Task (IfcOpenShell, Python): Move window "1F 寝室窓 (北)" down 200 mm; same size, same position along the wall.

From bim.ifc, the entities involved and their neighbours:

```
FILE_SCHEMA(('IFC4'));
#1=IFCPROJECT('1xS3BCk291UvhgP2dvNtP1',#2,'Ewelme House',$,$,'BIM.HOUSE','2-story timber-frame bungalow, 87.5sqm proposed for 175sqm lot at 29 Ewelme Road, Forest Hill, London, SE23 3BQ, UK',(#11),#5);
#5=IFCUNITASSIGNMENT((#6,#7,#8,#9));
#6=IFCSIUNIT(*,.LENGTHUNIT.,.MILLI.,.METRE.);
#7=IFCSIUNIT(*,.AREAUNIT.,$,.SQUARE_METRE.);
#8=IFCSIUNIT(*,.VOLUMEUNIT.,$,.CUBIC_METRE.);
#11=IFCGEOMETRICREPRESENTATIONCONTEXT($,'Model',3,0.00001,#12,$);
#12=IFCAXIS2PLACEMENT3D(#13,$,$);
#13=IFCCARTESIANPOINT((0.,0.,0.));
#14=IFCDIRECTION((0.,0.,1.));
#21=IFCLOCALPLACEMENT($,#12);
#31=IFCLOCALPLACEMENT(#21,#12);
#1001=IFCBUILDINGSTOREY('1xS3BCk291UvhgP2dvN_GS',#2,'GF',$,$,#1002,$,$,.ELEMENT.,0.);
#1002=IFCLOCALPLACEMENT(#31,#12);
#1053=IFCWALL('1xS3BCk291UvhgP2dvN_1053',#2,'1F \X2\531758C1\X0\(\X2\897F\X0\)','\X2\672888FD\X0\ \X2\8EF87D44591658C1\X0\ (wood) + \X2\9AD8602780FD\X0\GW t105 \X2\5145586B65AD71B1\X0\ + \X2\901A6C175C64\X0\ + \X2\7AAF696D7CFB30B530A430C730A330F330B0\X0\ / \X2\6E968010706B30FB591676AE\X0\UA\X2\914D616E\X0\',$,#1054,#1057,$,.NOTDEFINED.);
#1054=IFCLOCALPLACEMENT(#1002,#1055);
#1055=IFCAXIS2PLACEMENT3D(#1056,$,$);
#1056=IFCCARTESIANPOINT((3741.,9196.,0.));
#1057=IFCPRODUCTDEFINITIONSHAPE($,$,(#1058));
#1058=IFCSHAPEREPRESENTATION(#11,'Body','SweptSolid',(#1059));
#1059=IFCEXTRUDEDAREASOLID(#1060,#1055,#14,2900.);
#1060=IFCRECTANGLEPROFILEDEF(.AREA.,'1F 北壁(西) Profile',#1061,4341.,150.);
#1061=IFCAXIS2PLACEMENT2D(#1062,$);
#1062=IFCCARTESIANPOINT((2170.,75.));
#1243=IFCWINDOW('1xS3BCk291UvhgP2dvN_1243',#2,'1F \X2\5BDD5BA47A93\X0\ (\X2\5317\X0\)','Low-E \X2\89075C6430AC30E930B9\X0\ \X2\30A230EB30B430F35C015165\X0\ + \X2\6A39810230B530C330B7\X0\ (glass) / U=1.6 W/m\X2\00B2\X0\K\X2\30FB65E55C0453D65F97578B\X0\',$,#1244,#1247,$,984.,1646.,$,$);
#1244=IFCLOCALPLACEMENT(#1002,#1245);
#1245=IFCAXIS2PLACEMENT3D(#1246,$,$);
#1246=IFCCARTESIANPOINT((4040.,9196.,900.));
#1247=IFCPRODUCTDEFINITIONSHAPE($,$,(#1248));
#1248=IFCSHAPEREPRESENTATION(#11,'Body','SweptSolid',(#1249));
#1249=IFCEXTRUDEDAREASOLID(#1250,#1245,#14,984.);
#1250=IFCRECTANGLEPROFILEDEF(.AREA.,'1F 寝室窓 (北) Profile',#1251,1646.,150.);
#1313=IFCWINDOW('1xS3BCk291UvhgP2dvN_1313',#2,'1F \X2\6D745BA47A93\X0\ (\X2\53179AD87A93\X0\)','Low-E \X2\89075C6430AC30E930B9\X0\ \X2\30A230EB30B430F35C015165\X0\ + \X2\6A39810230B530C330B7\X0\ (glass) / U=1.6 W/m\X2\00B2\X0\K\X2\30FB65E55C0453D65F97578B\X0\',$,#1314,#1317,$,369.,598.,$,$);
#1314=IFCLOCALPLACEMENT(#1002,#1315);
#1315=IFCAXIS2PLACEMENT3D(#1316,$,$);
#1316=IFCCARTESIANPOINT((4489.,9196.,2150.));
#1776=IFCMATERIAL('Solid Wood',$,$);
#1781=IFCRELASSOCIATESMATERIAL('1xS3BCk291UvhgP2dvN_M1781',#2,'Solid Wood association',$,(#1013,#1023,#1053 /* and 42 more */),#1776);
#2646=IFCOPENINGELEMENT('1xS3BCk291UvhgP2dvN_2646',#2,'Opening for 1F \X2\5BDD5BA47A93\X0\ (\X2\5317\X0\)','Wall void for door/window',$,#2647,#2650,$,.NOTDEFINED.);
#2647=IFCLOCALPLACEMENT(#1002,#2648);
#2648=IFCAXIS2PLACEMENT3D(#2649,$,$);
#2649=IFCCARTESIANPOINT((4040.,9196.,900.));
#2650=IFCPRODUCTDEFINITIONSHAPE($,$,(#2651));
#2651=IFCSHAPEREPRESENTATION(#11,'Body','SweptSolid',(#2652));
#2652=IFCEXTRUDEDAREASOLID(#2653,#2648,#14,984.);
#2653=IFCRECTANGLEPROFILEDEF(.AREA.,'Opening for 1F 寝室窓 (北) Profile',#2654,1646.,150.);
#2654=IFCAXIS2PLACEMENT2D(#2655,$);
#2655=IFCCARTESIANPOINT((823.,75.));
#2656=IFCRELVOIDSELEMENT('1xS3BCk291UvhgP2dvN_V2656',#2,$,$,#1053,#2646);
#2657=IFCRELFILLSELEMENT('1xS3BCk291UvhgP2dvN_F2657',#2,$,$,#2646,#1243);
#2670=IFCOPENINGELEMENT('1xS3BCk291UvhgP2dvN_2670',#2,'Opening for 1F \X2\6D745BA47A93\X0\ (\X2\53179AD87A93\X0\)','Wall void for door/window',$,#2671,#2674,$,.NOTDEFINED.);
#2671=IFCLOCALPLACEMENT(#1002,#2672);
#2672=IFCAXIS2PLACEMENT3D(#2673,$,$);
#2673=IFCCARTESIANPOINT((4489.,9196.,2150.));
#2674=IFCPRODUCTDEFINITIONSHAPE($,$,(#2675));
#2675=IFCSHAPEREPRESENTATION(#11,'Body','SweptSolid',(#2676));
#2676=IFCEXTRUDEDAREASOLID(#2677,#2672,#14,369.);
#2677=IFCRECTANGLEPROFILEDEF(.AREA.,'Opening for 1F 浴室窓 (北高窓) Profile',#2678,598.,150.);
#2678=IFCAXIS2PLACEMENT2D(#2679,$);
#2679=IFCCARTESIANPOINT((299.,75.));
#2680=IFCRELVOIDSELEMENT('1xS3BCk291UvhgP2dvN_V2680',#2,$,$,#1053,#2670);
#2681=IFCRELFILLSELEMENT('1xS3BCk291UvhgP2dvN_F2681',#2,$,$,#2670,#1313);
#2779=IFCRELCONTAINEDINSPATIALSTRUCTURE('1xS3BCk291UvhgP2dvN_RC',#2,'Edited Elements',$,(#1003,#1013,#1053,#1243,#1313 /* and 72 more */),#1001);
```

```python
import numpy as np
import ifcopenshell
import ifcopenshell.api.geometry
import ifcopenshell.util.placement
import ifcopenshell.util.unit

model = ifcopenshell.open("bim.ifc")
unit_scale = ifcopenshell.util.unit.calculate_unit_scale(model)

window = model.by_guid("1xS3BCk291UvhgP2dvN_1243")
opening = window.FillsVoids[0].RelatingOpeningElement
dz = -200.0

shift = np.array([0.0, 0.0, dz])
# The window is not placed relative to its opening, so move both.
for product in (opening, window):
    matrix = ifcopenshell.util.placement.get_local_placement(product.ObjectPlacement)
    matrix[:3, 3] += shift
    ifcopenshell.api.geometry.edit_object_placement(model, product=product, matrix=matrix, is_si=False)

print(f"moved by {dz * unit_scale:+.3f} m")

model.write("bim_edited.ifc")
```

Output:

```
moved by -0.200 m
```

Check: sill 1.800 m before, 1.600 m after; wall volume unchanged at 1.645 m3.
